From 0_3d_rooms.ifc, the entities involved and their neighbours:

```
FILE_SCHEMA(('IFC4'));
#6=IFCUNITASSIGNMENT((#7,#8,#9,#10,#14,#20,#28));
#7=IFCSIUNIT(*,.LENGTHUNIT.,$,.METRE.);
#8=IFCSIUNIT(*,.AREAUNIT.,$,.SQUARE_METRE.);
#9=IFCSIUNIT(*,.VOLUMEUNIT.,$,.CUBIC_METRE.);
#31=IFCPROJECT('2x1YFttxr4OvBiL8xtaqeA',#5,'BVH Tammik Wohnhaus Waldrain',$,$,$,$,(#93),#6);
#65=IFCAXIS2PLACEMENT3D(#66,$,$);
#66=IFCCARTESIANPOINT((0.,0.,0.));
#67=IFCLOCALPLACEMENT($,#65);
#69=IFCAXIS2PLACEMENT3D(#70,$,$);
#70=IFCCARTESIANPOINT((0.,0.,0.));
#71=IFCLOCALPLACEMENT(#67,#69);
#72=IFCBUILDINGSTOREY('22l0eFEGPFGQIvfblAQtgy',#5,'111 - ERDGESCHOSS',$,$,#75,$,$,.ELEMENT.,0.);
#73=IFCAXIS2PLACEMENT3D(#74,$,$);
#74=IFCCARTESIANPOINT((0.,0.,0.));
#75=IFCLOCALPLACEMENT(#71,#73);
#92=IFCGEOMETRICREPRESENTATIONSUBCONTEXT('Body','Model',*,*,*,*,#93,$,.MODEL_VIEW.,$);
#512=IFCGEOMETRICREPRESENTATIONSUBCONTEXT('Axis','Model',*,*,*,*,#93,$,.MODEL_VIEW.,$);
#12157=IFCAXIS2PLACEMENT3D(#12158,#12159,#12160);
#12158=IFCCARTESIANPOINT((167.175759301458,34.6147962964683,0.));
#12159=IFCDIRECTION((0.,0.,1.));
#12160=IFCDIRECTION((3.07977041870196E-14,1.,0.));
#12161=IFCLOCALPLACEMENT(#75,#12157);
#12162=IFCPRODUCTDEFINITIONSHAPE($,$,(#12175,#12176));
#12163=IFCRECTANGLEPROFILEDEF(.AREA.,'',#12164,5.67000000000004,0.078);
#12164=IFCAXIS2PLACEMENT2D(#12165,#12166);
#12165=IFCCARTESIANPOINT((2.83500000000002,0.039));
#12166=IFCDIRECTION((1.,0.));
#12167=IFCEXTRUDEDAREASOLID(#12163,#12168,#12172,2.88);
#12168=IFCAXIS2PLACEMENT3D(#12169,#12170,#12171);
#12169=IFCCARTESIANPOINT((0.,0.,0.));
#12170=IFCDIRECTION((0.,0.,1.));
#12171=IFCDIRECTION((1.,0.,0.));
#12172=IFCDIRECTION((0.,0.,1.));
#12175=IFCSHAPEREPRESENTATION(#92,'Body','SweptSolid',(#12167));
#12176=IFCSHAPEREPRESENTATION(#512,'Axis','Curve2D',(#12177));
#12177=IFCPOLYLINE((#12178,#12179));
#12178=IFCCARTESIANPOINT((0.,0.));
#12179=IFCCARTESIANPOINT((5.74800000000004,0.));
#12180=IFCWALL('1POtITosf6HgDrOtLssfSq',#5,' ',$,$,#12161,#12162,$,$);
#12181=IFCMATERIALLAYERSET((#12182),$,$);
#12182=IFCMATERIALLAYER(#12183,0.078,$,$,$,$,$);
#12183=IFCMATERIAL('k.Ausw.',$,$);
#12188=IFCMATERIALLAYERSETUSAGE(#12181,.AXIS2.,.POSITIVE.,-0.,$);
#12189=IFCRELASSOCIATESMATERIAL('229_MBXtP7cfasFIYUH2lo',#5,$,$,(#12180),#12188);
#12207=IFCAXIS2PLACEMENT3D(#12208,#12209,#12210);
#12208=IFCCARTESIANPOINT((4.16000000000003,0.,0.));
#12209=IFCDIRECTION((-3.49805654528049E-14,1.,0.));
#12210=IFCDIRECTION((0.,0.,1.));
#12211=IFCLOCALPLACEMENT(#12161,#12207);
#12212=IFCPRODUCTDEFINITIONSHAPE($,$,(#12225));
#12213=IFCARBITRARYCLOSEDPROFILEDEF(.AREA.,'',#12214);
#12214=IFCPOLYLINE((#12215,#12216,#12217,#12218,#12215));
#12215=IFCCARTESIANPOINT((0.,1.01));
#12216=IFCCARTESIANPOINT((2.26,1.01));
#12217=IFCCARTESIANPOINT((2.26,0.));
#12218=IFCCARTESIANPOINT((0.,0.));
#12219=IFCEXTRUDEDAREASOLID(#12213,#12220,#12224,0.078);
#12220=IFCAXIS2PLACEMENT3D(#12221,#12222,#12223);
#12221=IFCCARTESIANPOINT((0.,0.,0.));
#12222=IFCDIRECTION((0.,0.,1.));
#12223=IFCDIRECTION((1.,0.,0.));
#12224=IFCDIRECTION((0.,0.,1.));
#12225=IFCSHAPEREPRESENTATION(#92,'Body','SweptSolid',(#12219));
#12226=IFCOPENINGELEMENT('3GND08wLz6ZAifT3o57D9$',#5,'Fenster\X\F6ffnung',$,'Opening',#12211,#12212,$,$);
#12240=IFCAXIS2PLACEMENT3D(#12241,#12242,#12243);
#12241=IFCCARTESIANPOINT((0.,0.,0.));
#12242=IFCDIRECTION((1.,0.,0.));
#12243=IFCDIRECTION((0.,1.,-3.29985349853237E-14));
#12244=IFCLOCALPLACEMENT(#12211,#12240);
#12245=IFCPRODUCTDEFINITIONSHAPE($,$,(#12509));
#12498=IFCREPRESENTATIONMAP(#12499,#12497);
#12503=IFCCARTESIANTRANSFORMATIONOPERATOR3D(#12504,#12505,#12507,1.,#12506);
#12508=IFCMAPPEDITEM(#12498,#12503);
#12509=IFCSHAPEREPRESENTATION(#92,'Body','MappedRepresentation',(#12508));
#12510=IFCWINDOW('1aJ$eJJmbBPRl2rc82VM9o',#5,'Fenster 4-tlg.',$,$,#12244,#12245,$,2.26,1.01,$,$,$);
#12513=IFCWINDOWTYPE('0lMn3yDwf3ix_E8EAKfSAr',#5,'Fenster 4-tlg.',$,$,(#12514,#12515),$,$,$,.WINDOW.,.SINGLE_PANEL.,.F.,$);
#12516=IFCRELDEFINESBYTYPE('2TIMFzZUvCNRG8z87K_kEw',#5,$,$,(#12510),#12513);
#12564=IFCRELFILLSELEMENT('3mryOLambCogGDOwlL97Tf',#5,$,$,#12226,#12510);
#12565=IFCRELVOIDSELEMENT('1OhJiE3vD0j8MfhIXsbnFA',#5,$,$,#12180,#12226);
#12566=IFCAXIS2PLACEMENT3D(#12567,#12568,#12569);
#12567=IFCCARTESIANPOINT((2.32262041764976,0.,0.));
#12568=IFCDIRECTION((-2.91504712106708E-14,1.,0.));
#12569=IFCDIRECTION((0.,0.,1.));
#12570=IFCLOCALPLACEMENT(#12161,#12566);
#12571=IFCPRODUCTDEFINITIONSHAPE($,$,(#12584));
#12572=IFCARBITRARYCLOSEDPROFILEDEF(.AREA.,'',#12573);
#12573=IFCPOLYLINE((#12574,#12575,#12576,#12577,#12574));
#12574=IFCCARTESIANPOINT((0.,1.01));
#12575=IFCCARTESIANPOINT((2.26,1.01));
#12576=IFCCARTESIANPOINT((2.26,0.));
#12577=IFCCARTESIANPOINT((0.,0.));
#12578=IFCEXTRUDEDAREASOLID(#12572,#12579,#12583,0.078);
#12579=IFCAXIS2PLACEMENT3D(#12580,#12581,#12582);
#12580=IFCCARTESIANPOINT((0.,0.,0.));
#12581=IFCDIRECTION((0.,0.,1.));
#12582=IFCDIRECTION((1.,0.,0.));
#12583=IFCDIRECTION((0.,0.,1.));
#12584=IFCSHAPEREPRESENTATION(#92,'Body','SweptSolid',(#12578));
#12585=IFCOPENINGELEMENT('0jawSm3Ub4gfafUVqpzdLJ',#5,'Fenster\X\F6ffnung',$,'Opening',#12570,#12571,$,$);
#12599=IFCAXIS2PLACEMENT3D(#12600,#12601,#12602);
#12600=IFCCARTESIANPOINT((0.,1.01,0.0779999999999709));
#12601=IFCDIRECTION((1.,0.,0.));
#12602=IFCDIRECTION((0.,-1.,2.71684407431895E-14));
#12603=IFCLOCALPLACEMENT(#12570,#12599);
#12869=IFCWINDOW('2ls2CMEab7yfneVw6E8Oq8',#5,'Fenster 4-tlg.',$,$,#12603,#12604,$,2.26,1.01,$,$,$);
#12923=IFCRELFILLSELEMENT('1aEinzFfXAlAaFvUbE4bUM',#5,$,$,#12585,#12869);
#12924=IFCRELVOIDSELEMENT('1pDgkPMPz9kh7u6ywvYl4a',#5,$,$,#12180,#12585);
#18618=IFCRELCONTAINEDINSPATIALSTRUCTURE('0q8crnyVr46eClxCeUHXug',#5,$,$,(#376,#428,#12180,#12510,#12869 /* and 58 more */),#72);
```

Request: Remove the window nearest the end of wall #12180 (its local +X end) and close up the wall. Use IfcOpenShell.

```python
import ifcopenshell
import ifcopenshell.api.feature
import ifcopenshell.api.root
import ifcopenshell.geom
import ifcopenshell.util.shape

model = ifcopenshell.open("0_3d_rooms.ifc")
settings = ifcopenshell.geom.settings()


def volume(element):
    """Net volume in cubic metres, openings subtracted."""
    shape = ifcopenshell.geom.create_shape(settings, element)
    return ifcopenshell.util.shape.get_volume(shape.geometry)


window = model.by_guid("1aJ$eJJmbBPRl2rc82VM9o")
opening = window.FillsVoids[0].RelatingOpeningElement
wall = opening.VoidsElements[0].RelatingBuildingElement
before = volume(wall)

ifcopenshell.api.root.remove_product(model, product=window)
ifcopenshell.api.feature.remove_feature(model, feature=opening)

after = volume(wall)

print(f"wall volume {before:.3f} -> {after:.3f} m3")

model.write("0_3d_rooms_v2.ifc")
```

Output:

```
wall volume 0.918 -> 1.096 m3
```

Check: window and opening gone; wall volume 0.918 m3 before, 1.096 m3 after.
